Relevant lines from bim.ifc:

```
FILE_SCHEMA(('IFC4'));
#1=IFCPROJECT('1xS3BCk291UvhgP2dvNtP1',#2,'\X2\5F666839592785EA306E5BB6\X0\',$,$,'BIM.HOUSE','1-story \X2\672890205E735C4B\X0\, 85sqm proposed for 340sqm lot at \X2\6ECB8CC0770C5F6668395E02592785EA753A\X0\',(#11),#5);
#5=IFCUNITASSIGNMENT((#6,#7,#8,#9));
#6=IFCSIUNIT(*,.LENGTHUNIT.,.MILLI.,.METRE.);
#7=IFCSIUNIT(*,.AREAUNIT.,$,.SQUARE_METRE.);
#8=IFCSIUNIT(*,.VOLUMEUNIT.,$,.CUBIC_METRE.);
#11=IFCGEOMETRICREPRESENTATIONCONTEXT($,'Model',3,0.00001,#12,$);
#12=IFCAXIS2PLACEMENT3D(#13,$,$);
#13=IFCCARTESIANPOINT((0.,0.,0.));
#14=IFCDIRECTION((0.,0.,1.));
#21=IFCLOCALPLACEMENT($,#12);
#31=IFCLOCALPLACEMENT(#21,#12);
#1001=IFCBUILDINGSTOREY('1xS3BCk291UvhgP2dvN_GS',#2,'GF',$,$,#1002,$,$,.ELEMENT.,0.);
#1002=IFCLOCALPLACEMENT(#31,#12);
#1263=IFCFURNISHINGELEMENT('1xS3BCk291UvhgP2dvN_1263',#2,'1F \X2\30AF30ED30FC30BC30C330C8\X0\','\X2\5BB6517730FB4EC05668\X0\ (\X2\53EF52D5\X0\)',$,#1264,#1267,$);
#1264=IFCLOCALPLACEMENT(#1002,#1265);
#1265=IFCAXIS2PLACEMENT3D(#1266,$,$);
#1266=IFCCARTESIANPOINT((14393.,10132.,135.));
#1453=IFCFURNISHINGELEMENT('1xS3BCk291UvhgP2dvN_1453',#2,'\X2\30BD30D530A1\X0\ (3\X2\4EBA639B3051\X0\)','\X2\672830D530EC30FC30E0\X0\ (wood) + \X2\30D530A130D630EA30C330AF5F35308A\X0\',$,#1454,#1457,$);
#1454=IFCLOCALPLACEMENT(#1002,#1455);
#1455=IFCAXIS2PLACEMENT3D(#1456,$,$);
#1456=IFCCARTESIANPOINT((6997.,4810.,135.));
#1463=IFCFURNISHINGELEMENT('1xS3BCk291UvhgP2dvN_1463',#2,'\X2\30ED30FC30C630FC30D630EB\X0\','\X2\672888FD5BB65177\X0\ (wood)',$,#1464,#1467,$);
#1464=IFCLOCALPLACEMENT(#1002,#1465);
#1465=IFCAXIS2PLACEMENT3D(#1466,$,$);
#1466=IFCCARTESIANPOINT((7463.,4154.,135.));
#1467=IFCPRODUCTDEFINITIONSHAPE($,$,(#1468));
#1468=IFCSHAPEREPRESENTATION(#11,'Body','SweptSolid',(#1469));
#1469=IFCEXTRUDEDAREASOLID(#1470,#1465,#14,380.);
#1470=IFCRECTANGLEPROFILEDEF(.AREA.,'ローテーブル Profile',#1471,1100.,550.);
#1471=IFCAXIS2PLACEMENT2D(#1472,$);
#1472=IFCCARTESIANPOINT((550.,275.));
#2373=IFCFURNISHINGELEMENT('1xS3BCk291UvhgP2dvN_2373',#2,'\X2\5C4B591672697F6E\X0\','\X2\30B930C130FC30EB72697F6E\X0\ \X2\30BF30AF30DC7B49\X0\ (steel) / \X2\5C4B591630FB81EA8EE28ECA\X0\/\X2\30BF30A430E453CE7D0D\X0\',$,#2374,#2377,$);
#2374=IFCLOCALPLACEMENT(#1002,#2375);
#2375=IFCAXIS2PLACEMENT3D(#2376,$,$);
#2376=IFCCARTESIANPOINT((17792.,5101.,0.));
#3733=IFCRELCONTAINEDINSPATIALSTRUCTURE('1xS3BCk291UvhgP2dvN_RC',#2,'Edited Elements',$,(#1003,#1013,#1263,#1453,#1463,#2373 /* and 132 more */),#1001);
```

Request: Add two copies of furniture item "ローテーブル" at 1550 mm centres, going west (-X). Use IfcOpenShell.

```python
import numpy as np
import ifcopenshell
import ifcopenshell.api.geometry
import ifcopenshell.api.root
import ifcopenshell.util.element
import ifcopenshell.util.placement
import ifcopenshell.util.unit

model = ifcopenshell.open("bim.ifc")
unit_scale = ifcopenshell.util.unit.calculate_unit_scale(model)


def reuse_history(source, copy):
    """copy_class also copies each property set's owner history, people and application; keep the originals."""
    for rel in copy.IsDefinedBy:
        if rel.is_a("IfcRelDefinesByProperties") and (history := rel.RelatingPropertyDefinition.OwnerHistory):
            rel.RelatingPropertyDefinition.OwnerHistory = source.OwnerHistory
            ifcopenshell.util.element.remove_deep2(model, history)


source = model.by_guid("1xS3BCk291UvhgP2dvN_1463")
base = ifcopenshell.util.placement.get_local_placement(source.ObjectPlacement)
step = np.array([-1.0, 0.0, 0.0]) * 1.55 / unit_scale

for i in range(1, 3):
    copy = ifcopenshell.api.root.copy_class(model, product=source)
    copy.Representation = ifcopenshell.util.element.copy_deep(
        model, source.Representation, exclude=["IfcGeometricRepresentationContext", "IfcRepresentationMap"]
    )
    reuse_history(source, copy)
    matrix = base.copy()
    matrix[:3, 3] += i * step
    print("added at", matrix[:3, 3].round(3) + 0.0)
    ifcopenshell.api.geometry.edit_object_placement(model, product=copy, matrix=matrix, is_si=False)

model.write("bim_edited.ifc")
```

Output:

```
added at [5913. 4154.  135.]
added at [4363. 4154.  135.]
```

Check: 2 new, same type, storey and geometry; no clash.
